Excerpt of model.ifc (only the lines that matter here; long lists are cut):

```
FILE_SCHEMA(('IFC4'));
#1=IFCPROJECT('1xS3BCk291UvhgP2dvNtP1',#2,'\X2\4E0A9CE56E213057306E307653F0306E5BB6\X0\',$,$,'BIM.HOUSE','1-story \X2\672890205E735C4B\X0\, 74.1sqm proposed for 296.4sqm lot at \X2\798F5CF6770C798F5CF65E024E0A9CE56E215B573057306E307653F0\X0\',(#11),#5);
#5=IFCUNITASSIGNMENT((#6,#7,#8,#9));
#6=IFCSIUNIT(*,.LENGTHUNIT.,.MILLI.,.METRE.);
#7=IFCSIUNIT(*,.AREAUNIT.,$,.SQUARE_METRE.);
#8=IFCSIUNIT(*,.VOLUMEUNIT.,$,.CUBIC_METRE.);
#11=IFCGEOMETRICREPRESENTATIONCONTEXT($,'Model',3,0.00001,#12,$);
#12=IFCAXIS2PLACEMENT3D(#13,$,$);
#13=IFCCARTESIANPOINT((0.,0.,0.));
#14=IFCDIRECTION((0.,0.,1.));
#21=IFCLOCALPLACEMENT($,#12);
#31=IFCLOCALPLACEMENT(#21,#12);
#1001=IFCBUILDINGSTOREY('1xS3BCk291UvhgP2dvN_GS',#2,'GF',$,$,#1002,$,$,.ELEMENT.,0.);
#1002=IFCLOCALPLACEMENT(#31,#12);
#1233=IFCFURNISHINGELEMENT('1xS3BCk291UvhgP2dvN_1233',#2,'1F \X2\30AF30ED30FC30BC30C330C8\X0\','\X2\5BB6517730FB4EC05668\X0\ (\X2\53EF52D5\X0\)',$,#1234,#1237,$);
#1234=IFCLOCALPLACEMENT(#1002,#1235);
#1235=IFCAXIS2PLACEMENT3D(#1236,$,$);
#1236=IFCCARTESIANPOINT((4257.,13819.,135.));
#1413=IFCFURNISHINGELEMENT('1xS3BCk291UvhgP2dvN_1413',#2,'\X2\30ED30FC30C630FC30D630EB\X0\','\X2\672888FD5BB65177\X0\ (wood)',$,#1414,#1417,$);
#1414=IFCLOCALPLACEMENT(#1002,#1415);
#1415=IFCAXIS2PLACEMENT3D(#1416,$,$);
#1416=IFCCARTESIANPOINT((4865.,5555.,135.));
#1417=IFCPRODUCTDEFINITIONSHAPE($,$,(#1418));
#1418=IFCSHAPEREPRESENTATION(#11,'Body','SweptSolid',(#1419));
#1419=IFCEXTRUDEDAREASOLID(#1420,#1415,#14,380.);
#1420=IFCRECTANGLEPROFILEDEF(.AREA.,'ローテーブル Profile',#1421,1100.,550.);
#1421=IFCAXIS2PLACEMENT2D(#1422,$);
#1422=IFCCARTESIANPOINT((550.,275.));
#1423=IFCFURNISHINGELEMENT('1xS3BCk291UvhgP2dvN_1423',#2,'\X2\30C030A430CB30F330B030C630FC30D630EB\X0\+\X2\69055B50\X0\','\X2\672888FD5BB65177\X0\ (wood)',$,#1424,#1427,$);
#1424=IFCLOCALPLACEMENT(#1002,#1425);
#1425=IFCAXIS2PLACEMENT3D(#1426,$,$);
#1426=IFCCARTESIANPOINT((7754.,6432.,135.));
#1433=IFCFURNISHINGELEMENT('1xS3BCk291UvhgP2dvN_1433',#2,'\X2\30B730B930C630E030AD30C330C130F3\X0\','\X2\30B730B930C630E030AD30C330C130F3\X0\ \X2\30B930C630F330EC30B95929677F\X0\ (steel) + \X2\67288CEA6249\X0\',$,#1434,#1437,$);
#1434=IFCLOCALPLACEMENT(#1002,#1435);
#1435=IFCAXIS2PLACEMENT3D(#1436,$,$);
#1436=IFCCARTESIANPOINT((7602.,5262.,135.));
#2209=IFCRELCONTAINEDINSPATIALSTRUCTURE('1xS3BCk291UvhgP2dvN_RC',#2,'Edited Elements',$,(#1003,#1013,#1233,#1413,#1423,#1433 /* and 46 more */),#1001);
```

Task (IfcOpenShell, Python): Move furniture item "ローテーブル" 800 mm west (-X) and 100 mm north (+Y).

```python
import ifcopenshell
import ifcopenshell.api.geometry
import ifcopenshell.util.placement

model = ifcopenshell.open("model.ifc")

item = model.by_guid("1xS3BCk291UvhgP2dvN_1413")
matrix = ifcopenshell.util.placement.get_local_placement(item.ObjectPlacement)
matrix[0, 3] -= 800.0
matrix[1, 3] += 100.0
ifcopenshell.api.geometry.edit_object_placement(model, product=item, matrix=matrix, is_si=False)

print(ifcopenshell.util.placement.get_local_placement(item.ObjectPlacement).round(3) + 0.0)

model.write("model_updated.ifc")
```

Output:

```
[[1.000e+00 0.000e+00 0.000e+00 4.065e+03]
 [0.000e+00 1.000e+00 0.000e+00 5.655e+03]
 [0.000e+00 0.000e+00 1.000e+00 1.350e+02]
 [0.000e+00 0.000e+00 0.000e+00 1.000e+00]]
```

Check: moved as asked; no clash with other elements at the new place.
